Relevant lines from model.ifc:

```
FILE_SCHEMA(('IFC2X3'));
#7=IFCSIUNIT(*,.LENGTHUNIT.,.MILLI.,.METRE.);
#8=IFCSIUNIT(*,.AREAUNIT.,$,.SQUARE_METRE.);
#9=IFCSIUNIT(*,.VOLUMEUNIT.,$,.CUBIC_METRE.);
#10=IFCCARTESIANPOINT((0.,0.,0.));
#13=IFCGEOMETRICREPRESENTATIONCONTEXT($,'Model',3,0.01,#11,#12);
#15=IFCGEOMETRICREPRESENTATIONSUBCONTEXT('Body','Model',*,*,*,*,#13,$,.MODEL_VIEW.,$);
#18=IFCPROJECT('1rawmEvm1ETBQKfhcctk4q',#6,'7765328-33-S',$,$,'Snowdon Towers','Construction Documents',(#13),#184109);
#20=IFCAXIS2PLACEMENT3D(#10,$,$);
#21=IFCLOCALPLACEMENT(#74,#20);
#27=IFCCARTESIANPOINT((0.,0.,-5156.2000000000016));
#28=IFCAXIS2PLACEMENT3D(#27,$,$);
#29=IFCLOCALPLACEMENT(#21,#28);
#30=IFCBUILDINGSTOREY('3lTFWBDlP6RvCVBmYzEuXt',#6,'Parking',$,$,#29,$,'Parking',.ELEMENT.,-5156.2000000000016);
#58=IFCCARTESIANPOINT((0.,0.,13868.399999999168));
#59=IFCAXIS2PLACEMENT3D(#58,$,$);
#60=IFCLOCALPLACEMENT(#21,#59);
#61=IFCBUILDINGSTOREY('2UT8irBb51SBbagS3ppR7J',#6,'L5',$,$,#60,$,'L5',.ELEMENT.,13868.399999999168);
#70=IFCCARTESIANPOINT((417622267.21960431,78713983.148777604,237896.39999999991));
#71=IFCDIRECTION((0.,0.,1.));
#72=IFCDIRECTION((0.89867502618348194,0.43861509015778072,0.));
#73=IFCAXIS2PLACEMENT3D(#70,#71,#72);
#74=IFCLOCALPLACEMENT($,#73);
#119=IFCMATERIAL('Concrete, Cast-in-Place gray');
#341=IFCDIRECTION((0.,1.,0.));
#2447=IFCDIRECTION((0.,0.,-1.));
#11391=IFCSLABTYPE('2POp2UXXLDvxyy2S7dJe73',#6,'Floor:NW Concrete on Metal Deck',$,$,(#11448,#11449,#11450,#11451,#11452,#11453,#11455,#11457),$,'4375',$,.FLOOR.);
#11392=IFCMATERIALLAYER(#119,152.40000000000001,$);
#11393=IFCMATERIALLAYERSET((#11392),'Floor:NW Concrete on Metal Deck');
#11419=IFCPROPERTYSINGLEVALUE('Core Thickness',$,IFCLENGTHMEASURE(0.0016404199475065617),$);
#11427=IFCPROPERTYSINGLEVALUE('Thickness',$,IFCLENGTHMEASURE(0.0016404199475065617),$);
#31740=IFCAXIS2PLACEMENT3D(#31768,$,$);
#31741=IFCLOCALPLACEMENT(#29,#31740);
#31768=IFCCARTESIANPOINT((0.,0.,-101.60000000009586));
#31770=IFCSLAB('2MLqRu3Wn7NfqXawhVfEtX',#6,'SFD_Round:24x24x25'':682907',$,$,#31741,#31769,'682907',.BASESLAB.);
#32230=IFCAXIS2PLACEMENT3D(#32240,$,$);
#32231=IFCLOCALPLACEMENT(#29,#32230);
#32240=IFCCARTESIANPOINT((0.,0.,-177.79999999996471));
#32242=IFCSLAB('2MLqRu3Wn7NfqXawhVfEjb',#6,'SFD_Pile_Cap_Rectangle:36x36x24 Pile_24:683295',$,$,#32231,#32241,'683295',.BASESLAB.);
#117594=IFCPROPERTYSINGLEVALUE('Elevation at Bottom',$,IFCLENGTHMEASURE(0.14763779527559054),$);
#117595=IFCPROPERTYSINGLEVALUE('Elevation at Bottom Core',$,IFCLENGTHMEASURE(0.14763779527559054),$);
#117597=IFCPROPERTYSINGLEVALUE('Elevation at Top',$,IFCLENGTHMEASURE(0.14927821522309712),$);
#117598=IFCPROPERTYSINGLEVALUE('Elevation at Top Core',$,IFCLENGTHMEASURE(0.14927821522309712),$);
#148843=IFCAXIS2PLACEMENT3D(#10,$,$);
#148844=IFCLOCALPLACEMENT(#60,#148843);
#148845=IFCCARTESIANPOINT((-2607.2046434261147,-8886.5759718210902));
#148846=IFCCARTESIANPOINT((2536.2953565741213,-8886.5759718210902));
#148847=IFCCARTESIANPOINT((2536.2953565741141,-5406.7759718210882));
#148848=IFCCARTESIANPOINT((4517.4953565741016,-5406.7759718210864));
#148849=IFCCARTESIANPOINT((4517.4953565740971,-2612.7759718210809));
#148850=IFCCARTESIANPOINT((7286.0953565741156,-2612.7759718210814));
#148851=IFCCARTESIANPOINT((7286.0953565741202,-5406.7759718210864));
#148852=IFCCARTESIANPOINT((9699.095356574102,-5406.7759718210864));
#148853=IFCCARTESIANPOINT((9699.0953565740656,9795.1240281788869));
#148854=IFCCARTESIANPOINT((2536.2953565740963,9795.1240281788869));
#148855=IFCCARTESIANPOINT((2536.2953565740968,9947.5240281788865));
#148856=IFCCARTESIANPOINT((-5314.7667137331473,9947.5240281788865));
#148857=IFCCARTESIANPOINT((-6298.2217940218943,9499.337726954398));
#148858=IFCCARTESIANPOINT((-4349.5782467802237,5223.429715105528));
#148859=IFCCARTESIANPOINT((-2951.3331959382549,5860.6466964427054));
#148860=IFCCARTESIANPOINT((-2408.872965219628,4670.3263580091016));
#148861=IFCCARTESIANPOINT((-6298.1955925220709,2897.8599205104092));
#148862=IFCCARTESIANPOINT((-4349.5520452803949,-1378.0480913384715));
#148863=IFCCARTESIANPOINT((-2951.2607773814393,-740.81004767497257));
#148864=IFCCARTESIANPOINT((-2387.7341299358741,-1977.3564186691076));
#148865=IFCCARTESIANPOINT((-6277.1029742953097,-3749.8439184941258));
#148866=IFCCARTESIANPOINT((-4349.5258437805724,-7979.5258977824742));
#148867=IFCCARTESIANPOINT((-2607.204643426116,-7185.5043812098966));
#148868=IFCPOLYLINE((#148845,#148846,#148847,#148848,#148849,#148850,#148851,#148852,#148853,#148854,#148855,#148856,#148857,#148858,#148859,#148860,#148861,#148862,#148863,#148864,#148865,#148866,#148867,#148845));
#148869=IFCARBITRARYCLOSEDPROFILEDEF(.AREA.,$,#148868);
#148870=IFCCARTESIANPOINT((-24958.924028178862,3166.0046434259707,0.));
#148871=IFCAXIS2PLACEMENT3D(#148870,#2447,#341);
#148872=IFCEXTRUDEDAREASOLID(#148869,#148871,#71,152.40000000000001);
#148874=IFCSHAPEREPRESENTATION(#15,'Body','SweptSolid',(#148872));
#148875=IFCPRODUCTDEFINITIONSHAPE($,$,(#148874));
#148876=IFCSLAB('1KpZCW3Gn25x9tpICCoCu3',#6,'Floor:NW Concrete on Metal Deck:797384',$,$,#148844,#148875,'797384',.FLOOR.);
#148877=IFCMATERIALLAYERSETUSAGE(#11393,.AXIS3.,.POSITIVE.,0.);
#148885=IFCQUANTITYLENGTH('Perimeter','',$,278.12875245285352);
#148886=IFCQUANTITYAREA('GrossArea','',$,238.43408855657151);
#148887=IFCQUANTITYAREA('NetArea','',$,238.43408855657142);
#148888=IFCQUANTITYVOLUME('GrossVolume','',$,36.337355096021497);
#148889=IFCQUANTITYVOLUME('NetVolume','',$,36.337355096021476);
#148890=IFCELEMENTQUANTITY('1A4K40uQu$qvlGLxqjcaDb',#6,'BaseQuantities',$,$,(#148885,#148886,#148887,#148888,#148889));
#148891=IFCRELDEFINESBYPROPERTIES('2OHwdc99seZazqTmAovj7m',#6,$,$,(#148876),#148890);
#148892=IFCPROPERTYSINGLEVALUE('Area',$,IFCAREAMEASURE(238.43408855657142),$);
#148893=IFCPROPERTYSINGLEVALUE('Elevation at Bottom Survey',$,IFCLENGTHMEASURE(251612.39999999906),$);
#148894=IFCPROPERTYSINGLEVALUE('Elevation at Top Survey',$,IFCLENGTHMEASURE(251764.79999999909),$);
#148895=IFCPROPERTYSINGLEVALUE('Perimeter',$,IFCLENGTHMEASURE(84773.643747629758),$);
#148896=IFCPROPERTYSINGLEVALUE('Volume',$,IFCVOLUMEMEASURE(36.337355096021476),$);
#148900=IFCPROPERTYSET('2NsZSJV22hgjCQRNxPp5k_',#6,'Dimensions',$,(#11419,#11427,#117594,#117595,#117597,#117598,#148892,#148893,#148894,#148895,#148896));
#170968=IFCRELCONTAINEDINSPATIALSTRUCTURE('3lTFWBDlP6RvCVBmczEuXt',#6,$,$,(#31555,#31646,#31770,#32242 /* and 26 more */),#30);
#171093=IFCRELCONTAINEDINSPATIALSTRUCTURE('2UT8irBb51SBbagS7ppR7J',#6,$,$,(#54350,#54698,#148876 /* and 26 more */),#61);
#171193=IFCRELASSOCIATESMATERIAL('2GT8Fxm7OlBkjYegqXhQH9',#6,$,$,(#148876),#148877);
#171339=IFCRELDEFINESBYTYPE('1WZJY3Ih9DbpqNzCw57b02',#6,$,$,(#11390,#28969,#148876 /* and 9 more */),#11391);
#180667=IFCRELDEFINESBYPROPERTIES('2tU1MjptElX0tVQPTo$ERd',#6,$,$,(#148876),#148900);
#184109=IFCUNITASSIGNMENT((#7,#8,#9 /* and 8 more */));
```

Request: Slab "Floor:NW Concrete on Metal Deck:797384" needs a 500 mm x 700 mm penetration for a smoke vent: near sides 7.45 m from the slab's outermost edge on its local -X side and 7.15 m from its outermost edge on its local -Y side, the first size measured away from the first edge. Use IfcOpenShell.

```python
import numpy as np
import ifcopenshell
import ifcopenshell.api.feature
import ifcopenshell.api.geometry
import ifcopenshell.api.pset
import ifcopenshell.api.root
import ifcopenshell.geom
import ifcopenshell.util.element
import ifcopenshell.util.placement
import ifcopenshell.util.representation
import ifcopenshell.util.shape
import ifcopenshell.util.unit

model = ifcopenshell.open("model.ifc")
unit_scale = ifcopenshell.util.unit.calculate_unit_scale(model)
area_scale = ifcopenshell.util.unit.calculate_unit_scale(model, "AREAUNIT")
volume_scale = ifcopenshell.util.unit.calculate_unit_scale(model, "VOLUMEUNIT")
settings = ifcopenshell.geom.settings()


def volume(element):
    """Net volume in cubic metres, openings subtracted."""
    shape = ifcopenshell.geom.create_shape(settings, element)
    return ifcopenshell.util.shape.get_volume(shape.geometry)


slab = model.by_guid("1KpZCW3Gn25x9tpICCoCu3")
before = volume(slab)

# Extent in the slab's own axes, in metres. The edges named are its -X and -Y sides.
slab_shape = ifcopenshell.geom.create_shape(settings, slab)
vertices = ifcopenshell.util.shape.get_vertices(slab_shape.geometry)
x_min, y_min, bottom = vertices.min(axis=0)
top = vertices[:, 2].max()

opening = ifcopenshell.api.root.create_entity(model, ifc_class="IfcOpeningElement", name="Smoke vent opening")
context = ifcopenshell.util.representation.get_context(model, "Model", "Body", "MODEL_VIEW")
width, depth = 0.5, 0.7
outline = [(0.0, 0.0), (width, 0.0), (width, depth), (0.0, depth), (0.0, 0.0)]
# Overshoot both faces by 50 mm so the cut is clean.
shape = ifcopenshell.api.geometry.add_slab_representation(
    model, context=context, depth=top - bottom + 0.1, polyline=outline
)
ifcopenshell.api.geometry.assign_representation(model, product=opening, representation=shape)

matrix = ifcopenshell.util.placement.get_local_placement(slab.ObjectPlacement)
matrix[:, 3] = matrix @ np.append(np.array([x_min + 7.45, y_min + 7.15, bottom - 0.05]) / unit_scale, 1.0)
ifcopenshell.api.geometry.edit_object_placement(model, product=opening, matrix=matrix, is_si=False)
ifcopenshell.api.feature.add_feature(model, feature=opening, element=slab)

after = volume(slab)

# Update the slab's stored quantities.
qto = model.by_id(ifcopenshell.util.element.get_pset(slab, "BaseQuantities", should_inherit=False)["id"])
ifcopenshell.api.pset.edit_qto(model, qto=qto, properties={
    "NetArea": after / (top - bottom) / area_scale,
    "NetVolume": after / volume_scale,
})
pset = model.by_id(ifcopenshell.util.element.get_pset(slab, "Dimensions", should_inherit=False)["id"])
ifcopenshell.api.pset.edit_pset(model, pset=pset, properties={
    "Area": model.create_entity("IfcAreaMeasure", after / (top - bottom) / area_scale),
    "Volume": model.create_entity("IfcVolumeMeasure", after / volume_scale),
})

print(f"slab volume {before:.3f} -> {after:.3f} m3")

model.write("model-out.ifc")
```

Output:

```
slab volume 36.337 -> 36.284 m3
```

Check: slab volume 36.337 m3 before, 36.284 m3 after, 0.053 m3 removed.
